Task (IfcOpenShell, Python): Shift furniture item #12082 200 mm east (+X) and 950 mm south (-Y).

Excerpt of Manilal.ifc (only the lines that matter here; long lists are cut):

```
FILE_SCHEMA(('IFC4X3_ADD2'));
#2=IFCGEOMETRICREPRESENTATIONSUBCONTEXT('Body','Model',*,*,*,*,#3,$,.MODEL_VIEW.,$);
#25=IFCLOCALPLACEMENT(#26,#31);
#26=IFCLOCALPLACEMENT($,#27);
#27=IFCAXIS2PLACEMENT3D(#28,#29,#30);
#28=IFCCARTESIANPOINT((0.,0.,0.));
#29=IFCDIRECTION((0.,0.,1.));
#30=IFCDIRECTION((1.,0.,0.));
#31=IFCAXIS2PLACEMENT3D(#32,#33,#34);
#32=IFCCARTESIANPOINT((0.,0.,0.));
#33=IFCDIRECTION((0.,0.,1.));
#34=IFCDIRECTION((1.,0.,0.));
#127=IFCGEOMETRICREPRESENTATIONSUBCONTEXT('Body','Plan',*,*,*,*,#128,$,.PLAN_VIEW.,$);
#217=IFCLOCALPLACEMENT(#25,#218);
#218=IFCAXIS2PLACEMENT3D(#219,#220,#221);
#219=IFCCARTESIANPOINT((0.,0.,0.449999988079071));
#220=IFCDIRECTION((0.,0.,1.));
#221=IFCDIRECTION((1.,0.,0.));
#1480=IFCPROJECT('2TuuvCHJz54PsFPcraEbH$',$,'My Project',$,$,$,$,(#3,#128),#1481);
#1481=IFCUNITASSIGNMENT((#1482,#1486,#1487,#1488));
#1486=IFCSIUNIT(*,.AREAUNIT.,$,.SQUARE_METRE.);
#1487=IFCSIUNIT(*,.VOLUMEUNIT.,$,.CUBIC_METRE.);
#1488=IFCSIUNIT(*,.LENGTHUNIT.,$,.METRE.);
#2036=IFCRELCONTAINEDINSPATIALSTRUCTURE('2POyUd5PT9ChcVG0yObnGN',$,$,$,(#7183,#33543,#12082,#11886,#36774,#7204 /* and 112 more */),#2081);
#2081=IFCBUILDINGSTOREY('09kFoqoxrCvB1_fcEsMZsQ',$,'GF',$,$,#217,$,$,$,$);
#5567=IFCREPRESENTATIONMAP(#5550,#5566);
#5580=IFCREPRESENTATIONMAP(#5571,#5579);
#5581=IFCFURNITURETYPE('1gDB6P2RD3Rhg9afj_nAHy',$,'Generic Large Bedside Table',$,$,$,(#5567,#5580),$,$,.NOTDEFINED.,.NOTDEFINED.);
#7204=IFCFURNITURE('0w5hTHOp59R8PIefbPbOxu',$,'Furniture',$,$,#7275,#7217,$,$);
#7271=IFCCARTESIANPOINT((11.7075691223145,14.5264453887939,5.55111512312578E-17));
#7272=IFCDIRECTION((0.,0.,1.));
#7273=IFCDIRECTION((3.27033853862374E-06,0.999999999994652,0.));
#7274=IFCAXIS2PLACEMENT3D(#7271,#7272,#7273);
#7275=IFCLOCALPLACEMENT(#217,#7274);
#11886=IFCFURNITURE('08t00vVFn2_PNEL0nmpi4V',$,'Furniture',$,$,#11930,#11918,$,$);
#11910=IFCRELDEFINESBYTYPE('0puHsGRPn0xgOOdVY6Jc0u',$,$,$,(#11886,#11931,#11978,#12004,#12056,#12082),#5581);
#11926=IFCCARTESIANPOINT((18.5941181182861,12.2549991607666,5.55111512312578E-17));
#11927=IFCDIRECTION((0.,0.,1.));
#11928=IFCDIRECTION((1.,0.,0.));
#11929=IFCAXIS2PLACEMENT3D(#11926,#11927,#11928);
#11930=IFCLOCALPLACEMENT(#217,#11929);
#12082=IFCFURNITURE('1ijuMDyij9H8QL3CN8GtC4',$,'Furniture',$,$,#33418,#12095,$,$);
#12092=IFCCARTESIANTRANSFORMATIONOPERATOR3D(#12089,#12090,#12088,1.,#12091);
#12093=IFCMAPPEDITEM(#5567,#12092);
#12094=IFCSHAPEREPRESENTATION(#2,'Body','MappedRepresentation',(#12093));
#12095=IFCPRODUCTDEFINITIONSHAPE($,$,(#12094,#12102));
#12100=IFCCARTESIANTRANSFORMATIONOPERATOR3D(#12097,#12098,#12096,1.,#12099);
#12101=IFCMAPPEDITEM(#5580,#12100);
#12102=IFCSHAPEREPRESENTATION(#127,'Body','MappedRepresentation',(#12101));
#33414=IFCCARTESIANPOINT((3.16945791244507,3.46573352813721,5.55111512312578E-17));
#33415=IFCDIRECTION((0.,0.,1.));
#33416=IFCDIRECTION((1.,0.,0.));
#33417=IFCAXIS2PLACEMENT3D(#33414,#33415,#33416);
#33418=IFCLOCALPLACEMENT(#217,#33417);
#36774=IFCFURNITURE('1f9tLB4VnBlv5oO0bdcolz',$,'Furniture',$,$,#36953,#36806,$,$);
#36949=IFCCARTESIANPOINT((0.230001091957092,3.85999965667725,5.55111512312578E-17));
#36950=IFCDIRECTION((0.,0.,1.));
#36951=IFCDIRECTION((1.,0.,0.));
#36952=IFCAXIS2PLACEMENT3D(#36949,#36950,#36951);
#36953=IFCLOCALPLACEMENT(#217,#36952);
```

```python
import ifcopenshell
import ifcopenshell.api.geometry
import ifcopenshell.util.placement
import ifcopenshell.util.unit

model = ifcopenshell.open("Manilal.ifc")
unit_scale = ifcopenshell.util.unit.calculate_unit_scale(model)

item = model.by_guid("1ijuMDyij9H8QL3CN8GtC4")
matrix = ifcopenshell.util.placement.get_local_placement(item.ObjectPlacement)
matrix[0, 3] += 0.2 / unit_scale
matrix[1, 3] -= 0.95 / unit_scale
ifcopenshell.api.geometry.edit_object_placement(model, product=item, matrix=matrix, is_si=False)

print(ifcopenshell.util.placement.get_local_placement(item.ObjectPlacement).round(3) + 0.0)

model.write("Manilal_updated.ifc")
```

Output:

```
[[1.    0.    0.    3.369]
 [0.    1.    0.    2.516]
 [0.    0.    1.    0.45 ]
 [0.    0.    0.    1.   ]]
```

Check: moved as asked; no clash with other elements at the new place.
